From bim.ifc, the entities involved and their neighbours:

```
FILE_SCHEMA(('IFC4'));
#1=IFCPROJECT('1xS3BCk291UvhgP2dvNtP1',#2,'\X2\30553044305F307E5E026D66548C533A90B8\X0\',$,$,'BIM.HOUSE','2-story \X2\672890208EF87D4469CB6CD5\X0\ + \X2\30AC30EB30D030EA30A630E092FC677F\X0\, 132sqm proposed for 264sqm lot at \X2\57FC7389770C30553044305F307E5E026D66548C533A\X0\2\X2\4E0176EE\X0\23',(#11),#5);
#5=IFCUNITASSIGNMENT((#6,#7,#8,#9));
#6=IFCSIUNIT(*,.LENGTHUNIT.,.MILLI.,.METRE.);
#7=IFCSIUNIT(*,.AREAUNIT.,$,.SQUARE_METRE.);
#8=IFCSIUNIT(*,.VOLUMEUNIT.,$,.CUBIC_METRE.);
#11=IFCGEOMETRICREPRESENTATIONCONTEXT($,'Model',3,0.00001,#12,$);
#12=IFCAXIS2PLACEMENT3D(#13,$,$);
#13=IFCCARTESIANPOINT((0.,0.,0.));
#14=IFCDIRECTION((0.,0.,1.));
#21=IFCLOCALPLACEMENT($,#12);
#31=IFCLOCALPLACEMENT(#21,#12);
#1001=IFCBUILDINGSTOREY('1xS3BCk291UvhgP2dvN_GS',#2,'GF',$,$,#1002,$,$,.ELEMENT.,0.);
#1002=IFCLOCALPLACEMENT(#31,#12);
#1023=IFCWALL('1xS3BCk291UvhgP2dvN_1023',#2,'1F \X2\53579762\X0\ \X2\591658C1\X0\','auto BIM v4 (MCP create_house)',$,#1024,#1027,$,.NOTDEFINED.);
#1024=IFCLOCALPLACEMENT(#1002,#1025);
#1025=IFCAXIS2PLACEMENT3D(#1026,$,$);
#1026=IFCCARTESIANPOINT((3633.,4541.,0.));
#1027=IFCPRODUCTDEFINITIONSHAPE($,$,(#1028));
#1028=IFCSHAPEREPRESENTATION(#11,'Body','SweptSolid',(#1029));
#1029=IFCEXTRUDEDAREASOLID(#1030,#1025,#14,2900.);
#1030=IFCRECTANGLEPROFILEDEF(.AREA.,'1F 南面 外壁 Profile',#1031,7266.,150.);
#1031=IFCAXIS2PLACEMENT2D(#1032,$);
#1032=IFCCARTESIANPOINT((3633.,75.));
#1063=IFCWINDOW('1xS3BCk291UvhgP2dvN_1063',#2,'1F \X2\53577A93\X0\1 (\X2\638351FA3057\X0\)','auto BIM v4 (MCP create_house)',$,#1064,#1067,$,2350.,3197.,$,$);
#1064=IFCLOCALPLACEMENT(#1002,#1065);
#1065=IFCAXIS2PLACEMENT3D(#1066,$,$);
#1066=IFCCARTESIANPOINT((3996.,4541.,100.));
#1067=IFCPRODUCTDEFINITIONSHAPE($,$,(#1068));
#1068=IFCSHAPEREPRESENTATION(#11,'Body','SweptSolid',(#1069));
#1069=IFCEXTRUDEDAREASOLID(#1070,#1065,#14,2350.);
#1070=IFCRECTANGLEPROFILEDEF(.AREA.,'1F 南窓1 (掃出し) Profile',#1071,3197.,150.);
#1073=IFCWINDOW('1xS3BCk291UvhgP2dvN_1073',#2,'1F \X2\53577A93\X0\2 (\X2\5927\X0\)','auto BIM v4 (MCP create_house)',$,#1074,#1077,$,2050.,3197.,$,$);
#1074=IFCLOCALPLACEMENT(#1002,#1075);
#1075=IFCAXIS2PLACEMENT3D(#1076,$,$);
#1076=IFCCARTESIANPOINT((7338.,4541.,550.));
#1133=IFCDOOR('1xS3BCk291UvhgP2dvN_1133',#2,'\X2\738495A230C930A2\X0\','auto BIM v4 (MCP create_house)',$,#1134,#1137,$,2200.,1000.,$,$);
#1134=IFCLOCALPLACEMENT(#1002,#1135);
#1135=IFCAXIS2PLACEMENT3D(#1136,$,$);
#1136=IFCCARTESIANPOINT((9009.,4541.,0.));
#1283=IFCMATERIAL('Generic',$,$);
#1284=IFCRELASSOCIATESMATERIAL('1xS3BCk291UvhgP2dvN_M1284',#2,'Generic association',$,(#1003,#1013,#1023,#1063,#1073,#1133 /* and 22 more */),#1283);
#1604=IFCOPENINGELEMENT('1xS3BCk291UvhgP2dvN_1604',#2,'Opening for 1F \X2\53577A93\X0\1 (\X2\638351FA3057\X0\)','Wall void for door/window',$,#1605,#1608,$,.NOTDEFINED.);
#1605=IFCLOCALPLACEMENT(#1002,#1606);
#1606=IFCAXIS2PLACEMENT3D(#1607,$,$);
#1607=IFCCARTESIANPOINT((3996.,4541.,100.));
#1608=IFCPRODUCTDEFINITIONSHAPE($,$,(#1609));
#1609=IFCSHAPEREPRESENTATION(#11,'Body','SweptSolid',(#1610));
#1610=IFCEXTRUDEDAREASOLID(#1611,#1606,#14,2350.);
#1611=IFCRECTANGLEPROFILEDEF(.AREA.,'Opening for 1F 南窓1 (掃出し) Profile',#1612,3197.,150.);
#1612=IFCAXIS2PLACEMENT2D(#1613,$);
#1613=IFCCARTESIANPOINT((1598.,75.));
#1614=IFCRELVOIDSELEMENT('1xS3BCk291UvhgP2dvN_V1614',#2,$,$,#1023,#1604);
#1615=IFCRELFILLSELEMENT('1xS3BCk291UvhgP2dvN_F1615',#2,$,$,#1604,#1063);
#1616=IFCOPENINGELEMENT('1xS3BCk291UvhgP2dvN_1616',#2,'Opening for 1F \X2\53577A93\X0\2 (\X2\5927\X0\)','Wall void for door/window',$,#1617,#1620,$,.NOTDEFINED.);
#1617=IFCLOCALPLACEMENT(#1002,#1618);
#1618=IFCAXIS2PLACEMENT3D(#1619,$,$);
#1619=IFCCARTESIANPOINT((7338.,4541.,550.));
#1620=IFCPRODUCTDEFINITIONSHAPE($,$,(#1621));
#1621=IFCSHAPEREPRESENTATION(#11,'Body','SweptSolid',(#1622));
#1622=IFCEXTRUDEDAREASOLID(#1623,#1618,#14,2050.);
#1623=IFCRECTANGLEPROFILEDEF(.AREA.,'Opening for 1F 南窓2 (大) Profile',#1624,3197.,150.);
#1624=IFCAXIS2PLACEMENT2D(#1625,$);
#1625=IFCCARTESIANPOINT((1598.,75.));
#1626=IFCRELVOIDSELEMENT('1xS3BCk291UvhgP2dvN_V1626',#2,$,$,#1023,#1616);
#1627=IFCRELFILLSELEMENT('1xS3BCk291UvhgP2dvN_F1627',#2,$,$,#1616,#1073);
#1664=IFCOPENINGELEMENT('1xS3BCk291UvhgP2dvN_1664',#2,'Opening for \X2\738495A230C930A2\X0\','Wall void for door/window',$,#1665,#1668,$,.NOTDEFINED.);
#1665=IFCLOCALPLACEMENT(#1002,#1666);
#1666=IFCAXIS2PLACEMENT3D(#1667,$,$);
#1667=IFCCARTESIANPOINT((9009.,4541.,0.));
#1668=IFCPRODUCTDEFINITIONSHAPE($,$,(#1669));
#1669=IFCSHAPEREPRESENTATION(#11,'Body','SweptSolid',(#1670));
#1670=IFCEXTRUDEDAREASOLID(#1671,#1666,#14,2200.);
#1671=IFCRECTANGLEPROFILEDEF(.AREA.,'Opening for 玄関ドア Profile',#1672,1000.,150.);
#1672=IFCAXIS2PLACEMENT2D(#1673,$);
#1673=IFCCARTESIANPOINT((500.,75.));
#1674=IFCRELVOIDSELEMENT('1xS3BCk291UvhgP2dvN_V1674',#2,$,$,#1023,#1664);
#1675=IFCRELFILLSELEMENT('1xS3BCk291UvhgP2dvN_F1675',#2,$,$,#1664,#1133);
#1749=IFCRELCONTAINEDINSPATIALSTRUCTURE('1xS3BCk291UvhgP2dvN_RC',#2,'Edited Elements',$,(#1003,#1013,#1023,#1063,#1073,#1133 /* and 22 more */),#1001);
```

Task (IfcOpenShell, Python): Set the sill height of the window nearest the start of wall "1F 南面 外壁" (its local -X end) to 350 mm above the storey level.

```python
import numpy as np
import ifcopenshell
import ifcopenshell.api.geometry
import ifcopenshell.geom
import ifcopenshell.util.element
import ifcopenshell.util.placement
import ifcopenshell.util.shape
import ifcopenshell.util.unit

model = ifcopenshell.open("bim.ifc")
unit_scale = ifcopenshell.util.unit.calculate_unit_scale(model)

window = model.by_guid("1xS3BCk291UvhgP2dvN_1063")
opening = window.FillsVoids[0].RelatingOpeningElement
storey = ifcopenshell.util.element.get_container(window, ifc_class="IfcBuildingStorey")
level = ifcopenshell.util.placement.get_local_placement(storey.ObjectPlacement)[2, 3]

# The opening's origin need not be at the sill, so measure its lowest point.
shape = ifcopenshell.geom.create_shape(ifcopenshell.geom.settings(), opening)
bottom = ifcopenshell.util.shape.get_shape_bottom_elevation(shape, shape.geometry) / unit_scale
dz = level + 0.35 / unit_scale - bottom

shift = np.array([0.0, 0.0, dz])
# The window is not placed relative to its opening, so move both.
for product in (opening, window):
    matrix = ifcopenshell.util.placement.get_local_placement(product.ObjectPlacement)
    matrix[:3, 3] += shift
    ifcopenshell.api.geometry.edit_object_placement(model, product=product, matrix=matrix, is_si=False)

print(f"moved by {dz * unit_scale:+.3f} m")

model.write("bim_edited.ifc")
```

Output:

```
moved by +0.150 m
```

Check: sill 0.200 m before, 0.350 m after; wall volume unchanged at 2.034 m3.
